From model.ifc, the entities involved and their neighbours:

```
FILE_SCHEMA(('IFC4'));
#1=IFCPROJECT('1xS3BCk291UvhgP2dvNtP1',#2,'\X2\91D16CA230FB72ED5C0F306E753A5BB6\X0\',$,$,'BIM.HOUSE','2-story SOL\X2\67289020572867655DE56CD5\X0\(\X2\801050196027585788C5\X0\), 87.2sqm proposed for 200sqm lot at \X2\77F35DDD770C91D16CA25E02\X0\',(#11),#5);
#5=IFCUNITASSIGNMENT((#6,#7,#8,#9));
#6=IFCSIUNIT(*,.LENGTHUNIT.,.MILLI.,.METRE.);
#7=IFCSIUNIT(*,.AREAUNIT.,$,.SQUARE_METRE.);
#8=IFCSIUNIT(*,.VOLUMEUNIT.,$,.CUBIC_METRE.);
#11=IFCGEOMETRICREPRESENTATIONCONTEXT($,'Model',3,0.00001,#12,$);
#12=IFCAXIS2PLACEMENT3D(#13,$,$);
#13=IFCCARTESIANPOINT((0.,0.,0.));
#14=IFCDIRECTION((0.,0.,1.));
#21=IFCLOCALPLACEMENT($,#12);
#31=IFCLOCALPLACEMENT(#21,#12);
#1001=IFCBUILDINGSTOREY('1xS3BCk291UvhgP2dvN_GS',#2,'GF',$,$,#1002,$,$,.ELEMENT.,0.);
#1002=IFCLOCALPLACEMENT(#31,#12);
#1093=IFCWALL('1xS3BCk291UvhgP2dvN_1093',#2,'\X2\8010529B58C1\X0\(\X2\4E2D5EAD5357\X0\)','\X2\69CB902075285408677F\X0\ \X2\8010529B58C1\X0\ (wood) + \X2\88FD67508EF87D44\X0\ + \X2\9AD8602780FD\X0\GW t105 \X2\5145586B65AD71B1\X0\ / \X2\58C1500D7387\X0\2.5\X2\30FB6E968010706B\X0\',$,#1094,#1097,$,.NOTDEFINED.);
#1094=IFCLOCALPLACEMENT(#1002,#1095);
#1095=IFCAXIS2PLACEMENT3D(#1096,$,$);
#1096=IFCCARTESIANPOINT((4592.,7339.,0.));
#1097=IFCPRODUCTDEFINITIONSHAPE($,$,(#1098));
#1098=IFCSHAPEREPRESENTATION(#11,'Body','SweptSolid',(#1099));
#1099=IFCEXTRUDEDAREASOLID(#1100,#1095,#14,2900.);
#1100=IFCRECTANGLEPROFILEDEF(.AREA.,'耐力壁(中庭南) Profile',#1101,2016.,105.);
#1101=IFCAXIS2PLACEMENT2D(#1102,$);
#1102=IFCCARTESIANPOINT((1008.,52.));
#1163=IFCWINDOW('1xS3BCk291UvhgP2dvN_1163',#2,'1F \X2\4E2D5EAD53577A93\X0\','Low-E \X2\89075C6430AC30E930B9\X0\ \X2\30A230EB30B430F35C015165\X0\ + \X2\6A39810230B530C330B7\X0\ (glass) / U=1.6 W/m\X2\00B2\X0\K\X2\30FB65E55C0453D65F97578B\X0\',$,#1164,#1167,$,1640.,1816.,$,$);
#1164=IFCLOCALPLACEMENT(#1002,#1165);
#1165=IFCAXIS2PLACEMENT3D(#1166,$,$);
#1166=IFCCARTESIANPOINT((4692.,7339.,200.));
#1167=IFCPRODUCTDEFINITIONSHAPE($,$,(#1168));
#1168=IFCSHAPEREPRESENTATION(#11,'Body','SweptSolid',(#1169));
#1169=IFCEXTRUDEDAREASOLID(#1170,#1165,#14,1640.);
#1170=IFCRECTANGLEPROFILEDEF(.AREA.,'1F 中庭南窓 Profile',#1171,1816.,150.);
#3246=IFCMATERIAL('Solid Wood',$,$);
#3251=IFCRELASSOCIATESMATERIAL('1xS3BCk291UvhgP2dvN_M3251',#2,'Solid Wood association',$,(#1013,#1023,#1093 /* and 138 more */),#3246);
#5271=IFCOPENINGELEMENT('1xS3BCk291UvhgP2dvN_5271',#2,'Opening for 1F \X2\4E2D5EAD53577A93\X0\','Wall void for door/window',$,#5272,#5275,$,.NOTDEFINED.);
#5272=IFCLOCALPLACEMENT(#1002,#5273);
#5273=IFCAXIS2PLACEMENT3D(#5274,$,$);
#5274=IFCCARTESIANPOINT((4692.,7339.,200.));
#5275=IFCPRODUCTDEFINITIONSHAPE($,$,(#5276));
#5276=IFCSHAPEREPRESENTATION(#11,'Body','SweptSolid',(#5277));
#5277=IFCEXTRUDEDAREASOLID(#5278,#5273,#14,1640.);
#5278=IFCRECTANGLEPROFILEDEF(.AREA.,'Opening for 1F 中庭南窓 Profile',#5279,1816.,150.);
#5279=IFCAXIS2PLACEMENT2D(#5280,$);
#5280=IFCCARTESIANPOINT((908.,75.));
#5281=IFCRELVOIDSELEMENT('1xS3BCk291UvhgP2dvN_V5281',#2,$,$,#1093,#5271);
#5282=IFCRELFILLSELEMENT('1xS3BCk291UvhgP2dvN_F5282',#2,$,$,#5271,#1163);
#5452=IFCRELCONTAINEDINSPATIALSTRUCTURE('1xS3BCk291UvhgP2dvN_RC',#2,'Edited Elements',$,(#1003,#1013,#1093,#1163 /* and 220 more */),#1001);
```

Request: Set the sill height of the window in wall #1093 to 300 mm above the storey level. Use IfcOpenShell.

```python
import numpy as np
import ifcopenshell
import ifcopenshell.api.geometry
import ifcopenshell.geom
import ifcopenshell.util.element
import ifcopenshell.util.placement
import ifcopenshell.util.shape
import ifcopenshell.util.unit

model = ifcopenshell.open("model.ifc")
unit_scale = ifcopenshell.util.unit.calculate_unit_scale(model)

window = model.by_id(1163)
opening = window.FillsVoids[0].RelatingOpeningElement
storey = ifcopenshell.util.element.get_container(window, ifc_class="IfcBuildingStorey")
level = ifcopenshell.util.placement.get_local_placement(storey.ObjectPlacement)[2, 3]

# The opening's origin need not be at the sill, so measure its lowest point.
shape = ifcopenshell.geom.create_shape(ifcopenshell.geom.settings(), opening)
bottom = ifcopenshell.util.shape.get_shape_bottom_elevation(shape, shape.geometry) / unit_scale
dz = level + 300.0 - bottom

shift = np.array([0.0, 0.0, dz])
# The window is not placed relative to its opening, so move both.
for product in (opening, window):
    matrix = ifcopenshell.util.placement.get_local_placement(product.ObjectPlacement)
    matrix[:3, 3] += shift
    ifcopenshell.api.geometry.edit_object_placement(model, product=product, matrix=matrix, is_si=False)

print(f"moved by {dz * unit_scale:+.3f} m")

model.write("model_rev.ifc")
```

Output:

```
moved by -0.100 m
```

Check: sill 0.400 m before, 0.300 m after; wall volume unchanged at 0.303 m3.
